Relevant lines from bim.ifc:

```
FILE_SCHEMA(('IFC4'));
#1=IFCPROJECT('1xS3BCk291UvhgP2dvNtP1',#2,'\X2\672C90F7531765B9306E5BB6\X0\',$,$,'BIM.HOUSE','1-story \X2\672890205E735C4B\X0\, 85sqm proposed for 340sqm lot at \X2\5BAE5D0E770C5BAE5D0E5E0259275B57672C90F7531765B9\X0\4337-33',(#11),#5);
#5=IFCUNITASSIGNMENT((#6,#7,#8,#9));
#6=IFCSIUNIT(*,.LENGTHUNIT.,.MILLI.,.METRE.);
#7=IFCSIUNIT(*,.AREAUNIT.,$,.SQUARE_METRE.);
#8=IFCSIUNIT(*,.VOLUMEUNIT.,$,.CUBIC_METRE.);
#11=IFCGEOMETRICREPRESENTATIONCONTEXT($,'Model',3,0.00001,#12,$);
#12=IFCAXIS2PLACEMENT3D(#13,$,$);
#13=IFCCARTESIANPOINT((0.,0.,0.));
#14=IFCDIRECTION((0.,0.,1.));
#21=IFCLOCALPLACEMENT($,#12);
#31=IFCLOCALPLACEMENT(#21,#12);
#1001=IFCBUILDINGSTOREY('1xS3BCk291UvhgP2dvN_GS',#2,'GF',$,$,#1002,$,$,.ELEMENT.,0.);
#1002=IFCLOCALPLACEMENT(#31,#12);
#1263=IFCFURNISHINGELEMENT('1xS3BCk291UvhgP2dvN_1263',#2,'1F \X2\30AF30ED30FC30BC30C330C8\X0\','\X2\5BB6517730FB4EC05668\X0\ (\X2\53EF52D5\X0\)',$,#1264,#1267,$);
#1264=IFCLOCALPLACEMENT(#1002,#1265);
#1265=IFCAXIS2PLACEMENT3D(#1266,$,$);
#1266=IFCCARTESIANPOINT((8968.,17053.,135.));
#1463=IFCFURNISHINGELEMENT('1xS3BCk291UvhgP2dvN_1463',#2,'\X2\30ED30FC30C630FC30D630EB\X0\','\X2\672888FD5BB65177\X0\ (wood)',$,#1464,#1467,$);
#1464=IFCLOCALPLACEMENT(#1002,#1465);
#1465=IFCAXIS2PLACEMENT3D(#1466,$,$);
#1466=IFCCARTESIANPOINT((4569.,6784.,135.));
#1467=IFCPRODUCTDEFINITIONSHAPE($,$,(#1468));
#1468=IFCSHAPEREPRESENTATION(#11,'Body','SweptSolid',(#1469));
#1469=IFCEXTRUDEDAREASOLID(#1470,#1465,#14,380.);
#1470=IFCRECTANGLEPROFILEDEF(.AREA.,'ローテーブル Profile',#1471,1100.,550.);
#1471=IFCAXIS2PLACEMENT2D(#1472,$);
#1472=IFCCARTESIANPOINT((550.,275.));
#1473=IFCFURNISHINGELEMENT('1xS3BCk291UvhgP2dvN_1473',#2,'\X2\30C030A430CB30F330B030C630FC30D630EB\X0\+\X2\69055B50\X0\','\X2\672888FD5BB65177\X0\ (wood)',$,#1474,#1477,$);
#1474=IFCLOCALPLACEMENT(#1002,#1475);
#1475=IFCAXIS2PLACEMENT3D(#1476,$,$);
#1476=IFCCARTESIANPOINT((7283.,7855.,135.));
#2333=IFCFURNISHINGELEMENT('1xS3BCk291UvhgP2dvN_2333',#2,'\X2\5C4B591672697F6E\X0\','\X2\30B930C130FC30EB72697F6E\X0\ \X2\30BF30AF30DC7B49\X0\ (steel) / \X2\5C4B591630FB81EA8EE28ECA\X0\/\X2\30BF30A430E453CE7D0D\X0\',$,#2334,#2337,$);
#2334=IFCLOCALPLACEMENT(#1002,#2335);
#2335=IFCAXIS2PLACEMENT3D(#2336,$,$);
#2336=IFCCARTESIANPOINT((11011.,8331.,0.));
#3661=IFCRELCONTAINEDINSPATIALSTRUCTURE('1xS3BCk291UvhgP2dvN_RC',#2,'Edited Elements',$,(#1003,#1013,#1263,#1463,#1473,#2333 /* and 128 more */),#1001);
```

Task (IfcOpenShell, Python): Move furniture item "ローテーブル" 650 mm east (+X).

```python
import ifcopenshell
import ifcopenshell.api.geometry
import ifcopenshell.util.placement
import ifcopenshell.util.unit

model = ifcopenshell.open("bim.ifc")
unit_scale = ifcopenshell.util.unit.calculate_unit_scale(model)

item = model.by_guid("1xS3BCk291UvhgP2dvN_1463")
matrix = ifcopenshell.util.placement.get_local_placement(item.ObjectPlacement)
matrix[0, 3] += 0.65 / unit_scale
ifcopenshell.api.geometry.edit_object_placement(model, product=item, matrix=matrix, is_si=False)

print(ifcopenshell.util.placement.get_local_placement(item.ObjectPlacement).round(3) + 0.0)

model.write("bim_v2.ifc")
```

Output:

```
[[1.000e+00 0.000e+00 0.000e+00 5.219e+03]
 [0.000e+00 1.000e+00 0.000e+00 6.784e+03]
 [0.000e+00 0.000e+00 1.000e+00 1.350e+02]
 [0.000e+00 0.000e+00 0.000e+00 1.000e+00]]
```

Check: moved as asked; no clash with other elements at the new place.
